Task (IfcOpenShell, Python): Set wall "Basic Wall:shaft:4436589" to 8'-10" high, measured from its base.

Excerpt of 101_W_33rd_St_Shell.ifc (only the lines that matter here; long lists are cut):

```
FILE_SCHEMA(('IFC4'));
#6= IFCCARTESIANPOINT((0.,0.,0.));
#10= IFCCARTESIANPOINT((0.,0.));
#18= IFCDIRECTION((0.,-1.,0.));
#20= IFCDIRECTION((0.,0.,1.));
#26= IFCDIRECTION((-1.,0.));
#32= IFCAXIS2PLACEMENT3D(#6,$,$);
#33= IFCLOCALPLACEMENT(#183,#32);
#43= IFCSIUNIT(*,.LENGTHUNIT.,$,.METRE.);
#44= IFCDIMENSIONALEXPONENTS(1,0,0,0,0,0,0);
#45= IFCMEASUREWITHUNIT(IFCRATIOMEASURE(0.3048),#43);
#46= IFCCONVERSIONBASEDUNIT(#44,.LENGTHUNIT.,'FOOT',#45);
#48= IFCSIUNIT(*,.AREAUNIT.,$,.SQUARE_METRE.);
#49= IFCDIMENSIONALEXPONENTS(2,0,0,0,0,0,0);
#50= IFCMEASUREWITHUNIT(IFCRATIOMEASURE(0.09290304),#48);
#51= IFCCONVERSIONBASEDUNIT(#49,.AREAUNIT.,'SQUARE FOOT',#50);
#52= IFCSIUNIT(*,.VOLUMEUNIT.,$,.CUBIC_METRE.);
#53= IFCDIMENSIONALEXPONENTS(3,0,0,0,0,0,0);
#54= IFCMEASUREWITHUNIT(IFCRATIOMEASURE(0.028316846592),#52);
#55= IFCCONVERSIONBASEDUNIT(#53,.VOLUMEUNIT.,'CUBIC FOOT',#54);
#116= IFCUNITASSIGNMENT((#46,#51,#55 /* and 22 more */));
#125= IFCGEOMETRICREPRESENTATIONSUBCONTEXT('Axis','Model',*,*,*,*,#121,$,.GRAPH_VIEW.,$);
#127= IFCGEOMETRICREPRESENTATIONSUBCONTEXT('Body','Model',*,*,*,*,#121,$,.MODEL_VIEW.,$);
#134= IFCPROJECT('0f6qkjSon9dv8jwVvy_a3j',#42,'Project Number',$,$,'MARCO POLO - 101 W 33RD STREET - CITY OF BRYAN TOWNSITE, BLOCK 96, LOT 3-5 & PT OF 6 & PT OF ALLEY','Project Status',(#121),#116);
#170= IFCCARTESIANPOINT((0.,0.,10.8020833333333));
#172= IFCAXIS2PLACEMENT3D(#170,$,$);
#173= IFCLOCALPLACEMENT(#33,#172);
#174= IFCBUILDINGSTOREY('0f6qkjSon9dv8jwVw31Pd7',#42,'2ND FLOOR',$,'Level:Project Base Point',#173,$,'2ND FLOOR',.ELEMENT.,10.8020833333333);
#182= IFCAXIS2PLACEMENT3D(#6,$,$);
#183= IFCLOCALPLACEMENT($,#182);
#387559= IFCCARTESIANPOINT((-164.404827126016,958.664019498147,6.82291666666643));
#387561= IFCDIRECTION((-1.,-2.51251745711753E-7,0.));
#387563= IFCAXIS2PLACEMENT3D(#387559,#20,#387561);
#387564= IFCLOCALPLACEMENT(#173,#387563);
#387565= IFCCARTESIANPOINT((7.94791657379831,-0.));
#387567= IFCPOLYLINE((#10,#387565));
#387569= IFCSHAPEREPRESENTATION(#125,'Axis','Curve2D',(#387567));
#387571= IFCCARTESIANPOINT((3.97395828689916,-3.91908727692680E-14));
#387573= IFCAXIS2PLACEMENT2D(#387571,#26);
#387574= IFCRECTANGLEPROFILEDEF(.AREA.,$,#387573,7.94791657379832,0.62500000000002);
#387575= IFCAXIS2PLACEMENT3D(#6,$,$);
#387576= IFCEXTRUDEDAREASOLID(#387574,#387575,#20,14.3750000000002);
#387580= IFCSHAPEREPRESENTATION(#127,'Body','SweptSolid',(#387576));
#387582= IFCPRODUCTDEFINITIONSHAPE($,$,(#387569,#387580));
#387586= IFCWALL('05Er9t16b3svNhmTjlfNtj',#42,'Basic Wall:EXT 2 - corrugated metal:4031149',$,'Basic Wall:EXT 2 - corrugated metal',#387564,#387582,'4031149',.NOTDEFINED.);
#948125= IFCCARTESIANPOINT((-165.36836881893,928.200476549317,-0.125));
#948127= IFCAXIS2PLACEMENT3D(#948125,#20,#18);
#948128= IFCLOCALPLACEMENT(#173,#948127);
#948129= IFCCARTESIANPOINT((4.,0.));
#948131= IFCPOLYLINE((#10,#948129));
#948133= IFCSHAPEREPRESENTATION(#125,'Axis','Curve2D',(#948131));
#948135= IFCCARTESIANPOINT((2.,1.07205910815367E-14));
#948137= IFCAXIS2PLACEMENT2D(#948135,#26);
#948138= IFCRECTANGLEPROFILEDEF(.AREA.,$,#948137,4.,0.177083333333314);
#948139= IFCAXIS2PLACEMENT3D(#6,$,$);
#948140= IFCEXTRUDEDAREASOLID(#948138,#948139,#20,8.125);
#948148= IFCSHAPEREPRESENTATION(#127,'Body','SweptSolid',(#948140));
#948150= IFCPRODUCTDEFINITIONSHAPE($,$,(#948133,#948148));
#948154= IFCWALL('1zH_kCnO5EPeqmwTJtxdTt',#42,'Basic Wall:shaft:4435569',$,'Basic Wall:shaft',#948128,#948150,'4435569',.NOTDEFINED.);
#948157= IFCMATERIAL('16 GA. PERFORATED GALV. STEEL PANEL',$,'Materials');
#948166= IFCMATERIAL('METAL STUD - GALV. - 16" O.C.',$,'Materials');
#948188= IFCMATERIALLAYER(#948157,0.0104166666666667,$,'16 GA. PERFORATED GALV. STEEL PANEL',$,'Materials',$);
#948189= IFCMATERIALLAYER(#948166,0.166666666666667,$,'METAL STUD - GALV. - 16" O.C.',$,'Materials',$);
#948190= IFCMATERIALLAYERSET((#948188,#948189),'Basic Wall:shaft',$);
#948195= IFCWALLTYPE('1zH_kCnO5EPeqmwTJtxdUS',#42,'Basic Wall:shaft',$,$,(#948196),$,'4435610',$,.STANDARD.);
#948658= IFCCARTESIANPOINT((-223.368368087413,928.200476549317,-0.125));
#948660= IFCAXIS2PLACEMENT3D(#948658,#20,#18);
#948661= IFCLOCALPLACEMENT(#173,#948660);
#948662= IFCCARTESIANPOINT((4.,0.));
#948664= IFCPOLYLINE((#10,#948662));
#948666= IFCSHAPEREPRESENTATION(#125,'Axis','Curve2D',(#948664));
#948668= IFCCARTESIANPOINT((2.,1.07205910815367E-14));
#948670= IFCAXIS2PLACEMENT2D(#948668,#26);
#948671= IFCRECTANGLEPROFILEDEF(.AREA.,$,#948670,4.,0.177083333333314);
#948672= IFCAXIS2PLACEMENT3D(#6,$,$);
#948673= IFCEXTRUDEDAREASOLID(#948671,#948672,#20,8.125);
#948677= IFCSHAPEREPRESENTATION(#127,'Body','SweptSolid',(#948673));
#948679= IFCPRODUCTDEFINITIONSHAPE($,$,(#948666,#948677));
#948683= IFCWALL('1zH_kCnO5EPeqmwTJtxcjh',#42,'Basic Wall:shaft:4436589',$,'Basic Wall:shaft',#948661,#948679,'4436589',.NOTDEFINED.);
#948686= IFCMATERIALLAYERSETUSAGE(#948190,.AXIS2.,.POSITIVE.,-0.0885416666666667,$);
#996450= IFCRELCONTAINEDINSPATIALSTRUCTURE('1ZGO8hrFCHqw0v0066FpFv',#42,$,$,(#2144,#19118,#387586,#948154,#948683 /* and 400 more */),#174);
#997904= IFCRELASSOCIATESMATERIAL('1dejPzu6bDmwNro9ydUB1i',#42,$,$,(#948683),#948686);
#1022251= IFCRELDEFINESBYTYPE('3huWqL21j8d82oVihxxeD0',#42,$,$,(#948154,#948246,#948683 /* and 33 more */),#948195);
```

```python
import ifcopenshell
import ifcopenshell.geom
import ifcopenshell.util.representation
import ifcopenshell.util.shape
import ifcopenshell.util.unit

model = ifcopenshell.open("101_W_33rd_St_Shell.ifc")
unit_scale = ifcopenshell.util.unit.calculate_unit_scale(model)
settings = ifcopenshell.geom.settings()


def volume(element):
    """Net volume in cubic metres, openings subtracted."""
    shape = ifcopenshell.geom.create_shape(settings, element)
    return ifcopenshell.util.shape.get_volume(shape.geometry)


wall = model.by_guid("1zH_kCnO5EPeqmwTJtxcjh")
before = volume(wall)

body = ifcopenshell.util.representation.get_representation(wall, "Model", "Body")
solid = body.Items[0]
old_height = solid.Depth
solid.Depth = 106 * 0.0254 / unit_scale
after = volume(wall)

print(f"height {old_height:g} -> {solid.Depth:g}, volume {before:.3f} -> {after:.3f} m3")

model.write("101_W_33rd_St_Shell_rev.ifc")
```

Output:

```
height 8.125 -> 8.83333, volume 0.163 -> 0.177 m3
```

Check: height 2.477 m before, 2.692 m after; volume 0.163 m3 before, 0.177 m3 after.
